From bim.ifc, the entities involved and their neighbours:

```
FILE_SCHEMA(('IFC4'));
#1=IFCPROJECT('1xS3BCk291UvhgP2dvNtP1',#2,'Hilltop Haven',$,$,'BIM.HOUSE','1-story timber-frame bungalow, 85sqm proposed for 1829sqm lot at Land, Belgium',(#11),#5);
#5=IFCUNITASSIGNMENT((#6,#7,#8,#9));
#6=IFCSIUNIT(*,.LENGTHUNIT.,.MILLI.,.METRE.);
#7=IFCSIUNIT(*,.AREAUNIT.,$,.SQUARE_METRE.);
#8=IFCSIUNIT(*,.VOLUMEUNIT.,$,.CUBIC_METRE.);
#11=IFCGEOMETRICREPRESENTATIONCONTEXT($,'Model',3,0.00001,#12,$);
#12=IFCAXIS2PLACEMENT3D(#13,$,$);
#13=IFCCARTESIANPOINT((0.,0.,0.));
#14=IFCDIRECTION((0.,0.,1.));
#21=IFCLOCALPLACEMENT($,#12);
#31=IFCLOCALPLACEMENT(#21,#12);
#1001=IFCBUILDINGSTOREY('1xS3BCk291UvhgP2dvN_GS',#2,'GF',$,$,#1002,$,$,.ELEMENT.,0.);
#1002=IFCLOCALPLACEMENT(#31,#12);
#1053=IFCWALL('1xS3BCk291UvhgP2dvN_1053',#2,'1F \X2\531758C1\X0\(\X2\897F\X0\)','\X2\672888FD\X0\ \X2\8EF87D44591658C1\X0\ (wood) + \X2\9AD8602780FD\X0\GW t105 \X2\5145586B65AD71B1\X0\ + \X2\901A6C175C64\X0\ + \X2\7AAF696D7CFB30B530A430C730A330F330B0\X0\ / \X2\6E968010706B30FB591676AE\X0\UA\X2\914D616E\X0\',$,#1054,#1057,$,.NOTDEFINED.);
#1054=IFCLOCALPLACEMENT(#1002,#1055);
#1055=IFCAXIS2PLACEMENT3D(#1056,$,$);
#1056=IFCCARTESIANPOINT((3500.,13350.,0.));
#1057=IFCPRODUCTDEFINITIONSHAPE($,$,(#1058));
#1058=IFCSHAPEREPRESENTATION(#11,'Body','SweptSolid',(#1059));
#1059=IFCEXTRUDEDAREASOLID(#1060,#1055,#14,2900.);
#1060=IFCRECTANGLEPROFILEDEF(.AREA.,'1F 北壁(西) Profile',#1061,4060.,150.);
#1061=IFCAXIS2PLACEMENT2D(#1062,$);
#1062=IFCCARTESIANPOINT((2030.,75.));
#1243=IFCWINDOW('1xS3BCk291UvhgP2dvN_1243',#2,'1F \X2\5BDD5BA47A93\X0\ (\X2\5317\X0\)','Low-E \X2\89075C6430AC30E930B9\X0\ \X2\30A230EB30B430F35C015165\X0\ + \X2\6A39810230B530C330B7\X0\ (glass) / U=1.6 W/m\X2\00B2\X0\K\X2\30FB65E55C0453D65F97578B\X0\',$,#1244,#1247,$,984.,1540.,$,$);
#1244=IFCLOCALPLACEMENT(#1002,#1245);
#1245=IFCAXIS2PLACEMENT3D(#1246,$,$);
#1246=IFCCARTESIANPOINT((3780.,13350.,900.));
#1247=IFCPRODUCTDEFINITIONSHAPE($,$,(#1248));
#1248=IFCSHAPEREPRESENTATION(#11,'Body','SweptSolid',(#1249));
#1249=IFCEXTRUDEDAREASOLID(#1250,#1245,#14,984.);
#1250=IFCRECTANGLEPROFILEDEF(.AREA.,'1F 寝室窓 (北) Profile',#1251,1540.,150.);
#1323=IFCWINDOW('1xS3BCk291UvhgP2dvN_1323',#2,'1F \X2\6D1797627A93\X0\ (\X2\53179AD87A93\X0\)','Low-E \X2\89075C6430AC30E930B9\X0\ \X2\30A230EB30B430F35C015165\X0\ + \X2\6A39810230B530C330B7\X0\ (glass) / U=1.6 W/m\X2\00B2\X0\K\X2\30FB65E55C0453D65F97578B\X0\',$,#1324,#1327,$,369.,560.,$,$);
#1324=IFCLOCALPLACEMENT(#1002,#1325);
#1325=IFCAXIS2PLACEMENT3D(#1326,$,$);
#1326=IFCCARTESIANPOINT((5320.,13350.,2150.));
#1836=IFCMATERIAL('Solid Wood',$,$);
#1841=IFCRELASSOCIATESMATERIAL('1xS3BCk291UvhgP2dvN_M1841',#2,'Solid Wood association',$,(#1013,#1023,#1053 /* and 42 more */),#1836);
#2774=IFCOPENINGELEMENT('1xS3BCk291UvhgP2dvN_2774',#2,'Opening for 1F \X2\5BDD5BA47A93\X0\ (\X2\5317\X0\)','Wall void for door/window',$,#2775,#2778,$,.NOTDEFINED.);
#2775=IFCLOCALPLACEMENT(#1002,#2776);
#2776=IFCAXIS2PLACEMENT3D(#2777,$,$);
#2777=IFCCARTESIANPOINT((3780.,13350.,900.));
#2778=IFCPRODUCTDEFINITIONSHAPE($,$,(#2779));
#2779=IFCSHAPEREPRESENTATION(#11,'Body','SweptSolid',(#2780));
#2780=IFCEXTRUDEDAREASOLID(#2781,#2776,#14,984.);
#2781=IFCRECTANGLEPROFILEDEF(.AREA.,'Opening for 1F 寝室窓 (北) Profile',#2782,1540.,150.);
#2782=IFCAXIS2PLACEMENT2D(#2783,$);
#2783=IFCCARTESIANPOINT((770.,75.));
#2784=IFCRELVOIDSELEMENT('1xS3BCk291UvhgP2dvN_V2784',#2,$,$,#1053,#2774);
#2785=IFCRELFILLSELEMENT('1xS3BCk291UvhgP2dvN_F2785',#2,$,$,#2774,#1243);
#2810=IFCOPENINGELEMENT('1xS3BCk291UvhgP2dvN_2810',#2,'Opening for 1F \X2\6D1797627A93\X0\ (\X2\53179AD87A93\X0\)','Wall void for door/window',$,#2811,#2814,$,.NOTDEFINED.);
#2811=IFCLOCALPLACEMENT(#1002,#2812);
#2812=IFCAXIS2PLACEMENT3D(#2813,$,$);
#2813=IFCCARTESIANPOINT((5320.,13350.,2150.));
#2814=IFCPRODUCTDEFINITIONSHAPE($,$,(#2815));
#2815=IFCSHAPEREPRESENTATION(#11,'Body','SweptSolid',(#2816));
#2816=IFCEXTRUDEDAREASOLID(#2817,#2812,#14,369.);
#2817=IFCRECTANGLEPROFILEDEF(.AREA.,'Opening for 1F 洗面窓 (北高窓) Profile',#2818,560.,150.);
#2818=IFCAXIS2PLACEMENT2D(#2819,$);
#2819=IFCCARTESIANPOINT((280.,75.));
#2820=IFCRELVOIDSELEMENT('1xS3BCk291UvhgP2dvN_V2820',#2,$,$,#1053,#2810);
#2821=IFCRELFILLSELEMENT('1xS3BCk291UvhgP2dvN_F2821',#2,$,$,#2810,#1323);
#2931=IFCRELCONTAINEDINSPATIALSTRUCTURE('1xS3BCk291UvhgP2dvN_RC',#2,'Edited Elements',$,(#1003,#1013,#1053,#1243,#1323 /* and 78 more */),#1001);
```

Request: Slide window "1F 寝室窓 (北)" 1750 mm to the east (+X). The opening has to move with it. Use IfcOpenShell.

```python
import ifcopenshell
import ifcopenshell.api.geometry
import ifcopenshell.util.placement
import ifcopenshell.util.unit

model = ifcopenshell.open("bim.ifc")
unit_scale = ifcopenshell.util.unit.calculate_unit_scale(model)

window = model.by_guid("1xS3BCk291UvhgP2dvN_1243")
opening = window.FillsVoids[0].RelatingOpeningElement
wall = opening.VoidsElements[0].RelatingBuildingElement

wall_matrix = ifcopenshell.util.placement.get_local_placement(wall.ObjectPlacement)
shift = wall_matrix[:3, 0] * 1.75 / unit_scale
before = ifcopenshell.util.placement.get_local_placement(window.ObjectPlacement)[:3, 3].copy()

# The window is not placed relative to its opening, so move both.
for product in (opening, window):
    matrix = ifcopenshell.util.placement.get_local_placement(product.ObjectPlacement)
    matrix[:3, 3] += shift
    ifcopenshell.api.geometry.edit_object_placement(model, product=product, matrix=matrix, is_si=False)

after = ifcopenshell.util.placement.get_local_placement(window.ObjectPlacement)[:3, 3]
print("window moved by", (after - before).round(3) + 0.0)

model.write("bim_v2.ifc")
```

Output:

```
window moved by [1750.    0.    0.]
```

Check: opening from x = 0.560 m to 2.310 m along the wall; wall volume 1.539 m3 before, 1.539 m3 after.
